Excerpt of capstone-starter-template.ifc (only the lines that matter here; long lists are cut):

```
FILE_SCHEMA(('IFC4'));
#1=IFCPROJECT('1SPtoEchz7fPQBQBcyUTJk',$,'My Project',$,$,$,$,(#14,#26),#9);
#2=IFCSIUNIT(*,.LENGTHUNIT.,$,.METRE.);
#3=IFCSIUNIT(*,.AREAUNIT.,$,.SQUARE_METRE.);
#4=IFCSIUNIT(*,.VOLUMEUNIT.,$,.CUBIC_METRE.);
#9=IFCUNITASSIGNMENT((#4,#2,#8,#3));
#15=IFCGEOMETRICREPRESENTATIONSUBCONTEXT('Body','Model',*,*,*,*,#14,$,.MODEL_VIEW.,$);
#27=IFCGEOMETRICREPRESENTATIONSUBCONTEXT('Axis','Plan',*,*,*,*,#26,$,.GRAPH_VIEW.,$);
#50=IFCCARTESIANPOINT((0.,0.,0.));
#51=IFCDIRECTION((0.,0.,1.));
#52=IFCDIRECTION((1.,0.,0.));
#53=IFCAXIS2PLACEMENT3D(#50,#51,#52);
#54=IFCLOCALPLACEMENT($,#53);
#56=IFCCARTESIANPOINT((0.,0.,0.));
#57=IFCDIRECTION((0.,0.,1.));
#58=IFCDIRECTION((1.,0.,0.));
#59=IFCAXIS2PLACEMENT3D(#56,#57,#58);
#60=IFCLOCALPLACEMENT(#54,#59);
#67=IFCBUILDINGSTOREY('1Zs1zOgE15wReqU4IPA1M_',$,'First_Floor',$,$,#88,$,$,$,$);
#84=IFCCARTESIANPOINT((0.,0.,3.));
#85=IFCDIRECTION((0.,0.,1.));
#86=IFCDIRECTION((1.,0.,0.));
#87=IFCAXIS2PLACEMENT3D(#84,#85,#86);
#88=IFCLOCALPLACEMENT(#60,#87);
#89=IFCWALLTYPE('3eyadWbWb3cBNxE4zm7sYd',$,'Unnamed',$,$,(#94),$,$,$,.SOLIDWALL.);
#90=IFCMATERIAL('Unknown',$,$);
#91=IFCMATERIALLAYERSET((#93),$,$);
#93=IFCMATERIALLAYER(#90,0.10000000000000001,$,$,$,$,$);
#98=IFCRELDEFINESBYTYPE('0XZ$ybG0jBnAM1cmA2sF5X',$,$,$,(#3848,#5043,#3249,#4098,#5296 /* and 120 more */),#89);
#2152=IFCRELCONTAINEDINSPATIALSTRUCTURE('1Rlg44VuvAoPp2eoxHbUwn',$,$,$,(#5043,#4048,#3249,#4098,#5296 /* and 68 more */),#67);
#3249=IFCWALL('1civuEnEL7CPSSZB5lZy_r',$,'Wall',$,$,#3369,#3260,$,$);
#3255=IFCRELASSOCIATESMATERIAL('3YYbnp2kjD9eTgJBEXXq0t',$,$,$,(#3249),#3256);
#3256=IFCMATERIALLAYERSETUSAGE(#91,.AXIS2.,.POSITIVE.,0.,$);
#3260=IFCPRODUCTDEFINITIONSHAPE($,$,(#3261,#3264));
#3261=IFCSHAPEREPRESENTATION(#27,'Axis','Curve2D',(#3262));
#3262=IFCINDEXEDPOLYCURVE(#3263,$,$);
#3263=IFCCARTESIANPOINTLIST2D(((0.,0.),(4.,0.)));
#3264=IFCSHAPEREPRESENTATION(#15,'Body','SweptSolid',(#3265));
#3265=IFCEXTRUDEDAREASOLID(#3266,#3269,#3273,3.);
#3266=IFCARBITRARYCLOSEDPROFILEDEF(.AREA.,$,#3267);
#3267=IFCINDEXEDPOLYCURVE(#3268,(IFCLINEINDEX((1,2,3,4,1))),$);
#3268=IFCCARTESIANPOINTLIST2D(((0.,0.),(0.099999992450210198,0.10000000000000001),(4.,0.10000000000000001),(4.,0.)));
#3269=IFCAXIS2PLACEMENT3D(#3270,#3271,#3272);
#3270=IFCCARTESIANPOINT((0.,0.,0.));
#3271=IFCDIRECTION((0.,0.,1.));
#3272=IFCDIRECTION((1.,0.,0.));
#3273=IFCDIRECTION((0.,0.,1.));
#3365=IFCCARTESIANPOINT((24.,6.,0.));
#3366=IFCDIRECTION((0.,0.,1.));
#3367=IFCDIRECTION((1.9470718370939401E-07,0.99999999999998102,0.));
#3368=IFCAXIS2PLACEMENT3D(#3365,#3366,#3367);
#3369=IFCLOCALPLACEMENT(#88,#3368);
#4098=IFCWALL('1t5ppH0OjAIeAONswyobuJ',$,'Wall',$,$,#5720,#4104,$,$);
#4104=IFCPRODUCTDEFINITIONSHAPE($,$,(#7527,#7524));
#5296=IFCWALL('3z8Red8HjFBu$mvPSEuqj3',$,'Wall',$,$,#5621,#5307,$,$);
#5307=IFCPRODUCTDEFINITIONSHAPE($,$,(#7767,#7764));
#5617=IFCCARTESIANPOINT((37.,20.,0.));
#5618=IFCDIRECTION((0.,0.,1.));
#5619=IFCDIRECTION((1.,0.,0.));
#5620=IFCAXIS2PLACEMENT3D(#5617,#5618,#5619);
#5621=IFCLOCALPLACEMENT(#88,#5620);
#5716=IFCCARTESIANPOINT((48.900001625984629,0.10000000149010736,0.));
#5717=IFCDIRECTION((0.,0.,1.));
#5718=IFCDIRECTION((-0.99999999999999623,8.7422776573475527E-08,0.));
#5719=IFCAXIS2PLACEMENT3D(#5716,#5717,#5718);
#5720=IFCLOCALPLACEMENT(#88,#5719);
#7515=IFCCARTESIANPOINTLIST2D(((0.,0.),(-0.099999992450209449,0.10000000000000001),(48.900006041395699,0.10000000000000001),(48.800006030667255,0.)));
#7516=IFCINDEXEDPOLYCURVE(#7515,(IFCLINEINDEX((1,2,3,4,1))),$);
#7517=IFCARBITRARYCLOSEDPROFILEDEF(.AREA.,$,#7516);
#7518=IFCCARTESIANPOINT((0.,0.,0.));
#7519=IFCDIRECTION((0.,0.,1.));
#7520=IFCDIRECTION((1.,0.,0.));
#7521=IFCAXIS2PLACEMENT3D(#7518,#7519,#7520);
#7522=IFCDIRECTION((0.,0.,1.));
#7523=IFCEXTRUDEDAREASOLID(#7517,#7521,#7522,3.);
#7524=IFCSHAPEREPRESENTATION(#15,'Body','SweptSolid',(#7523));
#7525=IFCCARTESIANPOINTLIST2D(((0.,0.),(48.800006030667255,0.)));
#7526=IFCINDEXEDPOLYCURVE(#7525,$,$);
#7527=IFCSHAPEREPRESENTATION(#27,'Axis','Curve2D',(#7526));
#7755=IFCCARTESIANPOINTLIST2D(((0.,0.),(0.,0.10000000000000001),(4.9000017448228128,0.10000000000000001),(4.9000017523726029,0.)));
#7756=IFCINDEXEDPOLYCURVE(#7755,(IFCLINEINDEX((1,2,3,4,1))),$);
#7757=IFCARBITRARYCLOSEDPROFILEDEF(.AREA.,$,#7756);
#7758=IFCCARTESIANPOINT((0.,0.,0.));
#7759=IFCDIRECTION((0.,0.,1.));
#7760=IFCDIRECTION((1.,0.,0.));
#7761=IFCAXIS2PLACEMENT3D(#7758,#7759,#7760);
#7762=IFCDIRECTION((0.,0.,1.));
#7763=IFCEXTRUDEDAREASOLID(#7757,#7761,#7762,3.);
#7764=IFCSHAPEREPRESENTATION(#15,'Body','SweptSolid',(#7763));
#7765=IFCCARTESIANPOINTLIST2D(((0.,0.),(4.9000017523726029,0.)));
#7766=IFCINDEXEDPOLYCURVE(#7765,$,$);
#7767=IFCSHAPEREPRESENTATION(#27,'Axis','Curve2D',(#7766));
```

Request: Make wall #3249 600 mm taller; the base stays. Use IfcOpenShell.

```python
import ifcopenshell
import ifcopenshell.geom
import ifcopenshell.util.representation
import ifcopenshell.util.shape
import ifcopenshell.util.unit

model = ifcopenshell.open("capstone-starter-template.ifc")
unit_scale = ifcopenshell.util.unit.calculate_unit_scale(model)
settings = ifcopenshell.geom.settings()


def volume(element):
    """Net volume in cubic metres, openings subtracted."""
    shape = ifcopenshell.geom.create_shape(settings, element)
    return ifcopenshell.util.shape.get_volume(shape.geometry)


wall = model.by_guid("1civuEnEL7CPSSZB5lZy_r")
before = volume(wall)

body = ifcopenshell.util.representation.get_representation(wall, "Model", "Body")
solid = body.Items[0]
old_height = solid.Depth
solid.Depth += 0.6 / unit_scale
after = volume(wall)

print(f"height {old_height:g} -> {solid.Depth:g}, volume {before:.3f} -> {after:.3f} m3")

model.write("capstone-starter-template_edited.ifc")
```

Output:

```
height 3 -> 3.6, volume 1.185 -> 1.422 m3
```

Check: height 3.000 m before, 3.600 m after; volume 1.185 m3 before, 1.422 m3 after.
